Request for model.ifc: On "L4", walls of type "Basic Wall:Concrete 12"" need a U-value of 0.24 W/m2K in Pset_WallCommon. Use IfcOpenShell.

First a look at what the model holds.

```python
import ifcopenshell
import ifcopenshell.util.element

model = ifcopenshell.open("model.ifc")
print(model.schema)
storey = next(s for s in model.by_type("IfcBuildingStorey") if s.Name == "L4")
walls = [e for e in ifcopenshell.util.element.get_decomposition(storey) if e.is_a("IfcWall")]
seen = {}
for e in walls:
    element_type = ifcopenshell.util.element.get_type(e)
    key = (element_type.Name if element_type != e and element_type else None, ifcopenshell.util.element.get_pset(e, "Pset_WallCommon", "ThermalTransmittance"))
    seen[key] = seen.get(key, 0) + 1
for (name, value), count in sorted(seen.items(), key=str):
    print(count, "x", name, "|", value)
```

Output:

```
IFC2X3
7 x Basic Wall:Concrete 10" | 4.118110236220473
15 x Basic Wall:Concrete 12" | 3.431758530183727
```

```python
import ifcopenshell
import ifcopenshell.api.pset
import ifcopenshell.util.element

model = ifcopenshell.open("model.ifc")

storey = next(s for s in model.by_type("IfcBuildingStorey") if s.Name == "L4")
walls = [e for e in ifcopenshell.util.element.get_decomposition(storey) if e.is_a("IfcWall")]

count = 0
for e in walls:
    element_type = ifcopenshell.util.element.get_type(e)
    if element_type in (None, e) or element_type.Name != 'Basic Wall:Concrete 12"':
        continue
    # add_pset returns the element's existing set when there is one.
    pset = ifcopenshell.api.pset.add_pset(model, product=e, name="Pset_WallCommon")
    ifcopenshell.api.pset.edit_pset(model, pset=pset, properties={"ThermalTransmittance": 0.24})
    count += 1

print(count, "walls updated")

model.write("model_updated.ifc")
```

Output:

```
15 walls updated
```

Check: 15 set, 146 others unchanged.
